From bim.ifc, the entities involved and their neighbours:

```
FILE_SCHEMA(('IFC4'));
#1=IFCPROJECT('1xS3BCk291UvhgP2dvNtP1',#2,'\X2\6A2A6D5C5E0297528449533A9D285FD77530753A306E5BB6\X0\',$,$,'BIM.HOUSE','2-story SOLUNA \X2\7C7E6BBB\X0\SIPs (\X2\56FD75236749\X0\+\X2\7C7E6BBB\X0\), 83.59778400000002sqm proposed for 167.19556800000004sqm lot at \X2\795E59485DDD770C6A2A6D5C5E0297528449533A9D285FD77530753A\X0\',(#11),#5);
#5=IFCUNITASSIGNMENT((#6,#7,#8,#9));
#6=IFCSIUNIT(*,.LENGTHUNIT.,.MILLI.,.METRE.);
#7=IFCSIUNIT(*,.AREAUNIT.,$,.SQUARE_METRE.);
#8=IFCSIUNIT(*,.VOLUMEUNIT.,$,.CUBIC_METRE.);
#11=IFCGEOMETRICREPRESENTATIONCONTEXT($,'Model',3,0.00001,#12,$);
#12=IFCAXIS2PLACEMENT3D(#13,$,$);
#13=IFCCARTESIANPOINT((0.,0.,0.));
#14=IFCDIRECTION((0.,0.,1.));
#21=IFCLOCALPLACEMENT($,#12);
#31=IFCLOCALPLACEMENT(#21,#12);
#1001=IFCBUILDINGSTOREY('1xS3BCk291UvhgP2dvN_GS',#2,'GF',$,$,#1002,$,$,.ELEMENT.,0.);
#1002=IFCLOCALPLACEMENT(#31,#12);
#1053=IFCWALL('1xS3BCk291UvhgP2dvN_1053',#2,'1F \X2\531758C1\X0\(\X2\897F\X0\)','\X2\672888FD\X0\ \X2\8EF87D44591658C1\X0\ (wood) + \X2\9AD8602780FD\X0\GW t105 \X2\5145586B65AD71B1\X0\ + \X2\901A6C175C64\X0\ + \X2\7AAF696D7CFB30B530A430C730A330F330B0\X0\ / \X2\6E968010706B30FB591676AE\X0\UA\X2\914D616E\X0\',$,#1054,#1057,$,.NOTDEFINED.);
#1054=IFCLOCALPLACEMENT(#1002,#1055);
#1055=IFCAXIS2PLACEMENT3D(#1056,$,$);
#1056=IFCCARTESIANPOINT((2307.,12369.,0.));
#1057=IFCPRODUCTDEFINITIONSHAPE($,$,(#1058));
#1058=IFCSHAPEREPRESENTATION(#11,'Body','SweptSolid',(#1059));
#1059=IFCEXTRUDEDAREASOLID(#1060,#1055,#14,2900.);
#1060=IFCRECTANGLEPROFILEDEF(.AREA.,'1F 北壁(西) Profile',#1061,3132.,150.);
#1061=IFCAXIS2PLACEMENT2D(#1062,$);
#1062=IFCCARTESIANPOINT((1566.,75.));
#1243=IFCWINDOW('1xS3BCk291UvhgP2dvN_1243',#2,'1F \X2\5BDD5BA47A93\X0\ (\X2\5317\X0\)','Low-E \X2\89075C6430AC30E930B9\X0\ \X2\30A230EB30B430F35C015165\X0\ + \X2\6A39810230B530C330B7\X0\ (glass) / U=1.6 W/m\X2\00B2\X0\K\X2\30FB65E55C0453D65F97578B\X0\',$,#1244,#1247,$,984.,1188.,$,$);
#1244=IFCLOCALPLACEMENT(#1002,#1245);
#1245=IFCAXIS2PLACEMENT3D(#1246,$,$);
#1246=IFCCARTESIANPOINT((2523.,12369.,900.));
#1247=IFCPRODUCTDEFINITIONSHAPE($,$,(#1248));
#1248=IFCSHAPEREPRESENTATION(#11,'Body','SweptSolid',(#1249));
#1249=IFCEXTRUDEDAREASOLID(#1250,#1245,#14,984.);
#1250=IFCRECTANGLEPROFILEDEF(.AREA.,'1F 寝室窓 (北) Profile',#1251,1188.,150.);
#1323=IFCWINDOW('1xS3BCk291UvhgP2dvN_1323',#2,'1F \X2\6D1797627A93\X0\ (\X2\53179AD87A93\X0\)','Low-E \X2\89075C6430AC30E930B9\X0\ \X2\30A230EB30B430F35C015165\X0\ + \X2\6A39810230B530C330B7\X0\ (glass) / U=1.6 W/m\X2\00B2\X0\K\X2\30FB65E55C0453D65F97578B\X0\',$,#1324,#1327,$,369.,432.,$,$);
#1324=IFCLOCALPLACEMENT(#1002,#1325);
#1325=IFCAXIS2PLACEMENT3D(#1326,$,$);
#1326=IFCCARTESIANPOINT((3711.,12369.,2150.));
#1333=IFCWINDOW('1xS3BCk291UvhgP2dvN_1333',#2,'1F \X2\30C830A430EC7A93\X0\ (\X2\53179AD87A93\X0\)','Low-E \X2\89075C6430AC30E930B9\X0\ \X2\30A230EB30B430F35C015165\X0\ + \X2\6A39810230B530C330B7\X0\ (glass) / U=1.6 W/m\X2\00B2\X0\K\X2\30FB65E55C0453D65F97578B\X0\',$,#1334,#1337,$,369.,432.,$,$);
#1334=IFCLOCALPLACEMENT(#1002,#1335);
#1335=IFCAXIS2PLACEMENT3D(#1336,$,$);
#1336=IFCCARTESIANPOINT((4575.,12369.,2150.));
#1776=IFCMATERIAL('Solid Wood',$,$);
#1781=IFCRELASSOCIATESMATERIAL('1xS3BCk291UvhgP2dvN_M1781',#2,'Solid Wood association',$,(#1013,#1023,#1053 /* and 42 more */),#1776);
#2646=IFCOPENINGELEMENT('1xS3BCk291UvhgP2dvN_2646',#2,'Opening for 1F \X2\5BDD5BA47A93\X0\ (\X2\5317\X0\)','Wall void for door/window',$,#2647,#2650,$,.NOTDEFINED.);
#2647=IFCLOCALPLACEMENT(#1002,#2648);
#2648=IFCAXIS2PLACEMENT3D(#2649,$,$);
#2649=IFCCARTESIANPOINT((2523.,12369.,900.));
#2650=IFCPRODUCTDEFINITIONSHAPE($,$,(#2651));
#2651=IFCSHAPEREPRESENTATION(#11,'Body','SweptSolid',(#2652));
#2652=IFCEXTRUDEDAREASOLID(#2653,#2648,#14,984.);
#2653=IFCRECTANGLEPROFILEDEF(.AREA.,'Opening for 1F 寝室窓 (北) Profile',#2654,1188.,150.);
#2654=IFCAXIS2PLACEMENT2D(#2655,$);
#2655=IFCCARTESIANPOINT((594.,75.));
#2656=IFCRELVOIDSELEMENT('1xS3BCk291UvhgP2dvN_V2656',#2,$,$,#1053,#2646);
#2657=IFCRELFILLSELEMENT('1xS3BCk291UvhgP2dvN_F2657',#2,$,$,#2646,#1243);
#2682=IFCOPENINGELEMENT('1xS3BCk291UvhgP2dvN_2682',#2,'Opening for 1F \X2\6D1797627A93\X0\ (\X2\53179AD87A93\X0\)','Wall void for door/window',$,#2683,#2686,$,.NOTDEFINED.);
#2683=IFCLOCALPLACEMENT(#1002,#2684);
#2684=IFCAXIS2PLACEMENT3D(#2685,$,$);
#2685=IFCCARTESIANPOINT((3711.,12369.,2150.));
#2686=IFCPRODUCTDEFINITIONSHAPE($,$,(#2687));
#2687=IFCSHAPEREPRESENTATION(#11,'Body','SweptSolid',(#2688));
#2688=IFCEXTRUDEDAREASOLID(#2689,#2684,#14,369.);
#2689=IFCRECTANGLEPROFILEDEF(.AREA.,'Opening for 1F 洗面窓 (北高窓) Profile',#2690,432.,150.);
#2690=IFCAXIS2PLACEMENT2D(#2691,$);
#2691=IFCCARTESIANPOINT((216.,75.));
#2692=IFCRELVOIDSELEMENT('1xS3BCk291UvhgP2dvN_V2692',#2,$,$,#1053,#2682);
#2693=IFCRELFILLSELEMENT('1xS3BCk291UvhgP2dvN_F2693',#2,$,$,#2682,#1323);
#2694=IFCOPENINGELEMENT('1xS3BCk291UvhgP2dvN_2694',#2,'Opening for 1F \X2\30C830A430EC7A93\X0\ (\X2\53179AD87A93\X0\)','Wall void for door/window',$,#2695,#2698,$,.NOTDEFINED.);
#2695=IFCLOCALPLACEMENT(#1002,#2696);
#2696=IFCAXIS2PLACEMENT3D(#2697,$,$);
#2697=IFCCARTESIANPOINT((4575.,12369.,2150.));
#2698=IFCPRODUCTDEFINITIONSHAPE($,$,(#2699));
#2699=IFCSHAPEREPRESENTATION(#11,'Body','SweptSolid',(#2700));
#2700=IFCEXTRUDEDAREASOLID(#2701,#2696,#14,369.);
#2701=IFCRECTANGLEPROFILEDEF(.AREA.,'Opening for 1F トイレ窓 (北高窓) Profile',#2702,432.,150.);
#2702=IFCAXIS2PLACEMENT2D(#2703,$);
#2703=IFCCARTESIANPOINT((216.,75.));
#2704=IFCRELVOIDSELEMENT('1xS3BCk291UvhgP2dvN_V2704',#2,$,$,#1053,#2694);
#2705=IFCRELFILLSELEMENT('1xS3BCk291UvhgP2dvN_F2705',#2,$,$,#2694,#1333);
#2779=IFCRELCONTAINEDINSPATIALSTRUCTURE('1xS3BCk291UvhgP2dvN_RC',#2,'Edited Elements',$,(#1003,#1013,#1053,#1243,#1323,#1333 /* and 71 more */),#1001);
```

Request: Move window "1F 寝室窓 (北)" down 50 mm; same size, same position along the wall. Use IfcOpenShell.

```python
import numpy as np
import ifcopenshell
import ifcopenshell.api.geometry
import ifcopenshell.util.placement
import ifcopenshell.util.unit

model = ifcopenshell.open("bim.ifc")
unit_scale = ifcopenshell.util.unit.calculate_unit_scale(model)

window = model.by_guid("1xS3BCk291UvhgP2dvN_1243")
opening = window.FillsVoids[0].RelatingOpeningElement
dz = -0.05 / unit_scale

shift = np.array([0.0, 0.0, dz])
# The window is not placed relative to its opening, so move both.
for product in (opening, window):
    matrix = ifcopenshell.util.placement.get_local_placement(product.ObjectPlacement)
    matrix[:3, 3] += shift
    ifcopenshell.api.geometry.edit_object_placement(model, product=product, matrix=matrix, is_si=False)

print(f"moved by {dz * unit_scale:+.3f} m")

model.write("bim_rev.ifc")
```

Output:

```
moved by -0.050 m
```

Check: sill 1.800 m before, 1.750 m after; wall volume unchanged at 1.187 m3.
